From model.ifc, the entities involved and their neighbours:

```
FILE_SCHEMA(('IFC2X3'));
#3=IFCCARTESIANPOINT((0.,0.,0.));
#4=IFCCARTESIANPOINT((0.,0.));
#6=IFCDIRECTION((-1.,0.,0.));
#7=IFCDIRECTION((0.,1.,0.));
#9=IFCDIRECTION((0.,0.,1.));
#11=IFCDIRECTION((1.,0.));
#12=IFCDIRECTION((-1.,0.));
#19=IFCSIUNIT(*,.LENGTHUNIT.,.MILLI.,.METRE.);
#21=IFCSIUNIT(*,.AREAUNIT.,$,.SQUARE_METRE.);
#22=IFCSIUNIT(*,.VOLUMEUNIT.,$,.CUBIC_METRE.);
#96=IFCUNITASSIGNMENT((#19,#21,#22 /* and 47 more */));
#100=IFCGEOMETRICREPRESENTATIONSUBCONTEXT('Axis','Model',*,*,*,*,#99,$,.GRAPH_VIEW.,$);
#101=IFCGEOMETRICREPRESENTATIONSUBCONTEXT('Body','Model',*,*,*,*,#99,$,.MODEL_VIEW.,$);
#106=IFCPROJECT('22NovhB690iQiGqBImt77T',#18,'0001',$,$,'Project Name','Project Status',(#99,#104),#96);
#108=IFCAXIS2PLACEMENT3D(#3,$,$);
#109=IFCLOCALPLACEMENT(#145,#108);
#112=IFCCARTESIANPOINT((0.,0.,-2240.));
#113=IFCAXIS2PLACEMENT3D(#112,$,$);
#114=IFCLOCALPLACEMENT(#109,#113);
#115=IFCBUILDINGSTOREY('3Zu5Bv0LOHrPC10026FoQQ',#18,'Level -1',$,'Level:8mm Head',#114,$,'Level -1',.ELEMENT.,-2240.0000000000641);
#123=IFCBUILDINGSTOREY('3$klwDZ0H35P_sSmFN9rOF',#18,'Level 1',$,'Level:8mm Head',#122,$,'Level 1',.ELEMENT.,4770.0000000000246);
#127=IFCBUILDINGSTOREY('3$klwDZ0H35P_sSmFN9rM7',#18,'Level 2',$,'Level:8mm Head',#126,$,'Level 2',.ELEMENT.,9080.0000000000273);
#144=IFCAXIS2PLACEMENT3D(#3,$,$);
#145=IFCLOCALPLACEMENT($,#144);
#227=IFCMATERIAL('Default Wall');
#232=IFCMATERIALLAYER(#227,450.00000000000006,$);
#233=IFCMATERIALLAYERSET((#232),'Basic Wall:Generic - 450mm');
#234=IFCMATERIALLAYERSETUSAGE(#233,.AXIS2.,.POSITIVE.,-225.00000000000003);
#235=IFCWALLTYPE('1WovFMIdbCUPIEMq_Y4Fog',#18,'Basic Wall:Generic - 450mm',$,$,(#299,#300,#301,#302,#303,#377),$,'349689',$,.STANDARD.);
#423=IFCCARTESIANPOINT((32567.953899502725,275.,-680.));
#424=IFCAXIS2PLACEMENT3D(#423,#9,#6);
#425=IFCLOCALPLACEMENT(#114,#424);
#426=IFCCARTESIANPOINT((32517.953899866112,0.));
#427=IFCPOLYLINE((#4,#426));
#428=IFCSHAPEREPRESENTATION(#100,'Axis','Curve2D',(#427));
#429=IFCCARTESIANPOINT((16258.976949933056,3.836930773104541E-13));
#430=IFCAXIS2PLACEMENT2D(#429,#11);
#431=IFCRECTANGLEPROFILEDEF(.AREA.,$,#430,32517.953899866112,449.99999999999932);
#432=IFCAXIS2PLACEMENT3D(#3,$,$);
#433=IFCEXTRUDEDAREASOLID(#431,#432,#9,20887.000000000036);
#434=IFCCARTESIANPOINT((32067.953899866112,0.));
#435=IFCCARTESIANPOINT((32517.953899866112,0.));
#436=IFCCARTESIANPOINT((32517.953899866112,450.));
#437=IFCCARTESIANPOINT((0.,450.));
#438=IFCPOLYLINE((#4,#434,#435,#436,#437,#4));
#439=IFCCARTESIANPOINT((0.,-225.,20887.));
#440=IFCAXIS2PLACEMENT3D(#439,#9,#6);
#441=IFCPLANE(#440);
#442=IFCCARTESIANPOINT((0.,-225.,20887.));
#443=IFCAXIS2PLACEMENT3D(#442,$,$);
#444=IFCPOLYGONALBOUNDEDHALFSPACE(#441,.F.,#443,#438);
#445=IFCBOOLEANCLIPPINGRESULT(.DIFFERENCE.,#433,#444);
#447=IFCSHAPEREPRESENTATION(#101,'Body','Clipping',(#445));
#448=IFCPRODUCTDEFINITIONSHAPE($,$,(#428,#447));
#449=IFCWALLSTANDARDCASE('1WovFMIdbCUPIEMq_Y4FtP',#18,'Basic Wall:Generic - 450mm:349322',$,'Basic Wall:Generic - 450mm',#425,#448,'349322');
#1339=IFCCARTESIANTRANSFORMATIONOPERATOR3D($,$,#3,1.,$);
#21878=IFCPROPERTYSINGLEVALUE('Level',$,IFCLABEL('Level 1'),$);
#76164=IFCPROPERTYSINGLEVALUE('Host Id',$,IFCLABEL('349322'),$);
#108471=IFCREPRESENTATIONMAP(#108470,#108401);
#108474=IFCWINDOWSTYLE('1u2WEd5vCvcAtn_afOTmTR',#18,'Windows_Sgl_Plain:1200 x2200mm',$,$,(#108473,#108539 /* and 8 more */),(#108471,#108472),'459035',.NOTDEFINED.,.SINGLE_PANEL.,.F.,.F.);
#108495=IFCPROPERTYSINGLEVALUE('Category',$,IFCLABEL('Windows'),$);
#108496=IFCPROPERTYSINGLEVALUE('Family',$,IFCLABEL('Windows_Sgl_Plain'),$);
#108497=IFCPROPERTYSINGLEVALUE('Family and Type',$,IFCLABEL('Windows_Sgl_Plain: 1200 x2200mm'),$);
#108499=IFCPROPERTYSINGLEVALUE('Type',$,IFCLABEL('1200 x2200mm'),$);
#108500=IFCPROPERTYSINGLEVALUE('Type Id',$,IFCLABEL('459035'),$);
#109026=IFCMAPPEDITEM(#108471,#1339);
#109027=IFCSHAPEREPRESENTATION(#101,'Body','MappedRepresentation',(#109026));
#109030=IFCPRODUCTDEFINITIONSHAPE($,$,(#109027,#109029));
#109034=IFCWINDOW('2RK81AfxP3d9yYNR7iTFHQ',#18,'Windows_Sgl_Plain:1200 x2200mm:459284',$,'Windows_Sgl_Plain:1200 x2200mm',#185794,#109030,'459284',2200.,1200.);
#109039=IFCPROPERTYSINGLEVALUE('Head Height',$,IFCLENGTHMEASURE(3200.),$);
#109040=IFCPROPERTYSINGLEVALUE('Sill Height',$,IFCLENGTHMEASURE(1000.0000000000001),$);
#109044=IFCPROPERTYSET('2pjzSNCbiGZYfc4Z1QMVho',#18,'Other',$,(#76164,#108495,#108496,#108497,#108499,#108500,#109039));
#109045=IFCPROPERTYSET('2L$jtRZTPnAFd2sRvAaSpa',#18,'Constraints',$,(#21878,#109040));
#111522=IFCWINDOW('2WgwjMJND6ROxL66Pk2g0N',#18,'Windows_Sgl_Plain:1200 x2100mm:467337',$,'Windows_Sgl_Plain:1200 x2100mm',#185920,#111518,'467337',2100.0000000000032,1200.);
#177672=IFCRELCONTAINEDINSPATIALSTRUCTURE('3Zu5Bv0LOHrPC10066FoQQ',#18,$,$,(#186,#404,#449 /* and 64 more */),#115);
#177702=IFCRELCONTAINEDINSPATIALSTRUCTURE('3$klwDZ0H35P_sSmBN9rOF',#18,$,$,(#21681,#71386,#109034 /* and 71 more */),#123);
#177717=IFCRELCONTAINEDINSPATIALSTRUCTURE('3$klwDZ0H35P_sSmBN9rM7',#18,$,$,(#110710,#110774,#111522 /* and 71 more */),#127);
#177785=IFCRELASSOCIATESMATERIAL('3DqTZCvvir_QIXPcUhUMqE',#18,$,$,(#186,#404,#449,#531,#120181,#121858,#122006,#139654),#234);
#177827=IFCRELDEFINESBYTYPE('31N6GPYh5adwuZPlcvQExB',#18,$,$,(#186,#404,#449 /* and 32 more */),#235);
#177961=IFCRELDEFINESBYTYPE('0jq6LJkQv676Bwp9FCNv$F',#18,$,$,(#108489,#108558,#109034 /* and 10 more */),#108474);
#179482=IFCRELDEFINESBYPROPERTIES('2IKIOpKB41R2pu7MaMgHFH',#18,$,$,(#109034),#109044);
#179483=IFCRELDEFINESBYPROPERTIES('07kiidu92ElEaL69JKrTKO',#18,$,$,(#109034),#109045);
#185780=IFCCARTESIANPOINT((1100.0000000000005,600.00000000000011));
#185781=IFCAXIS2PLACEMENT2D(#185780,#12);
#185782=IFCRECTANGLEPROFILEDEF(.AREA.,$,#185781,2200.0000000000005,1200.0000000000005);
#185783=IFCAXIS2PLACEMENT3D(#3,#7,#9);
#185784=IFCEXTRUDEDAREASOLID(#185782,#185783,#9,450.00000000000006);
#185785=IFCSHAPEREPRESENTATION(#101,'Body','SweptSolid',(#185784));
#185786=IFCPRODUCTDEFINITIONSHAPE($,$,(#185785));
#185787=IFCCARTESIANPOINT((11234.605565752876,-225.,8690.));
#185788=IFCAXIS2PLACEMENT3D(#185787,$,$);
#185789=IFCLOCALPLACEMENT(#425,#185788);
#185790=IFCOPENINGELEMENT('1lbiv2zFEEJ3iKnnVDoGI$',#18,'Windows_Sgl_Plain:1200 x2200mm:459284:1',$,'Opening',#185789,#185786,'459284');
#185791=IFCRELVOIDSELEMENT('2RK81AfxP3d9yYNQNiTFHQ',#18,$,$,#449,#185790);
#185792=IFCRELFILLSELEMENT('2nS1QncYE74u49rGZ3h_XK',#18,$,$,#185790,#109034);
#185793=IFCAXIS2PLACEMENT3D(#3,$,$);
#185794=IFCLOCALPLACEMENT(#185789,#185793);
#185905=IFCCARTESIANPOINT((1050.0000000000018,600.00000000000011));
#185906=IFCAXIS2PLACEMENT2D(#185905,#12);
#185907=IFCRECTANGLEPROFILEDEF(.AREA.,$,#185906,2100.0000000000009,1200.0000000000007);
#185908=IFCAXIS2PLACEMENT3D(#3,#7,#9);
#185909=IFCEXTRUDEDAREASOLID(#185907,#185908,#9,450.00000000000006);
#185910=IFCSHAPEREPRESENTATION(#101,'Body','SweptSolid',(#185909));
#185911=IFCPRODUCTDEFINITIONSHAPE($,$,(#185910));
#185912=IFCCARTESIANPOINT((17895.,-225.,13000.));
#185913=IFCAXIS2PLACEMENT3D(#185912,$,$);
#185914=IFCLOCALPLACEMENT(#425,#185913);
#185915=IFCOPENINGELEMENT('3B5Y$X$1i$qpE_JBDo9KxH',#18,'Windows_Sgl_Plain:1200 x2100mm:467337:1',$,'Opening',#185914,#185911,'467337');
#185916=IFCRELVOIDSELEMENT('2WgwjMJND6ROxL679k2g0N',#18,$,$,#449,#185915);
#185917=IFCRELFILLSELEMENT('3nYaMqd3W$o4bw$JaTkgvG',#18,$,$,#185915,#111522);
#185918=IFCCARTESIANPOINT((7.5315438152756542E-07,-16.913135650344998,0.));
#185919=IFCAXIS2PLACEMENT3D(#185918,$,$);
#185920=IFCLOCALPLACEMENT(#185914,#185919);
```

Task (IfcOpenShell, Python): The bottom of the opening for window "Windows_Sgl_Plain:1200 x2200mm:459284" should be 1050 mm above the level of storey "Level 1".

```python
import numpy as np
import ifcopenshell
import ifcopenshell.api.geometry
import ifcopenshell.api.pset
import ifcopenshell.geom
import ifcopenshell.util.element
import ifcopenshell.util.placement
import ifcopenshell.util.shape
import ifcopenshell.util.unit

model = ifcopenshell.open("model.ifc")
unit_scale = ifcopenshell.util.unit.calculate_unit_scale(model)

window = model.by_guid("2RK81AfxP3d9yYNR7iTFHQ")
opening = window.FillsVoids[0].RelatingOpeningElement
storey = ifcopenshell.util.element.get_container(window, ifc_class="IfcBuildingStorey")
level = ifcopenshell.util.placement.get_local_placement(storey.ObjectPlacement)[2, 3]

# The opening's origin need not be at the sill, so measure its lowest point.
shape = ifcopenshell.geom.create_shape(ifcopenshell.geom.settings(), opening)
bottom = ifcopenshell.util.shape.get_shape_bottom_elevation(shape, shape.geometry) / unit_scale
dz = level + 1050.0 - bottom

shift = np.array([0.0, 0.0, dz])
# The window is placed relative to its opening, so it follows when the opening moves.
matrix = ifcopenshell.util.placement.get_local_placement(opening.ObjectPlacement)
matrix[:3, 3] += shift
ifcopenshell.api.geometry.edit_object_placement(
    model, product=opening, matrix=matrix, is_si=False, should_transform_children=True
)

# Keep the stored heights in step.
pset = model.by_id(ifcopenshell.util.element.get_pset(window, "Other", should_inherit=False)["id"])
ifcopenshell.api.pset.edit_pset(model, pset=pset, properties={
    "Head Height": model.create_entity("IfcLengthMeasure", ifcopenshell.util.element.get_pset(window, "Other", "Head Height") + dz),
})
pset = model.by_id(ifcopenshell.util.element.get_pset(window, "Constraints", should_inherit=False)["id"])
ifcopenshell.api.pset.edit_pset(model, pset=pset, properties={
    "Sill Height": model.create_entity("IfcLengthMeasure", ifcopenshell.util.element.get_pset(window, "Constraints", "Sill Height") + dz),
})

print(f"moved by {dz * unit_scale:+.3f} m")

model.write("model_rev.ifc")
```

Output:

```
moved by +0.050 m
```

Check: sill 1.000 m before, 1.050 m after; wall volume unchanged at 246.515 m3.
